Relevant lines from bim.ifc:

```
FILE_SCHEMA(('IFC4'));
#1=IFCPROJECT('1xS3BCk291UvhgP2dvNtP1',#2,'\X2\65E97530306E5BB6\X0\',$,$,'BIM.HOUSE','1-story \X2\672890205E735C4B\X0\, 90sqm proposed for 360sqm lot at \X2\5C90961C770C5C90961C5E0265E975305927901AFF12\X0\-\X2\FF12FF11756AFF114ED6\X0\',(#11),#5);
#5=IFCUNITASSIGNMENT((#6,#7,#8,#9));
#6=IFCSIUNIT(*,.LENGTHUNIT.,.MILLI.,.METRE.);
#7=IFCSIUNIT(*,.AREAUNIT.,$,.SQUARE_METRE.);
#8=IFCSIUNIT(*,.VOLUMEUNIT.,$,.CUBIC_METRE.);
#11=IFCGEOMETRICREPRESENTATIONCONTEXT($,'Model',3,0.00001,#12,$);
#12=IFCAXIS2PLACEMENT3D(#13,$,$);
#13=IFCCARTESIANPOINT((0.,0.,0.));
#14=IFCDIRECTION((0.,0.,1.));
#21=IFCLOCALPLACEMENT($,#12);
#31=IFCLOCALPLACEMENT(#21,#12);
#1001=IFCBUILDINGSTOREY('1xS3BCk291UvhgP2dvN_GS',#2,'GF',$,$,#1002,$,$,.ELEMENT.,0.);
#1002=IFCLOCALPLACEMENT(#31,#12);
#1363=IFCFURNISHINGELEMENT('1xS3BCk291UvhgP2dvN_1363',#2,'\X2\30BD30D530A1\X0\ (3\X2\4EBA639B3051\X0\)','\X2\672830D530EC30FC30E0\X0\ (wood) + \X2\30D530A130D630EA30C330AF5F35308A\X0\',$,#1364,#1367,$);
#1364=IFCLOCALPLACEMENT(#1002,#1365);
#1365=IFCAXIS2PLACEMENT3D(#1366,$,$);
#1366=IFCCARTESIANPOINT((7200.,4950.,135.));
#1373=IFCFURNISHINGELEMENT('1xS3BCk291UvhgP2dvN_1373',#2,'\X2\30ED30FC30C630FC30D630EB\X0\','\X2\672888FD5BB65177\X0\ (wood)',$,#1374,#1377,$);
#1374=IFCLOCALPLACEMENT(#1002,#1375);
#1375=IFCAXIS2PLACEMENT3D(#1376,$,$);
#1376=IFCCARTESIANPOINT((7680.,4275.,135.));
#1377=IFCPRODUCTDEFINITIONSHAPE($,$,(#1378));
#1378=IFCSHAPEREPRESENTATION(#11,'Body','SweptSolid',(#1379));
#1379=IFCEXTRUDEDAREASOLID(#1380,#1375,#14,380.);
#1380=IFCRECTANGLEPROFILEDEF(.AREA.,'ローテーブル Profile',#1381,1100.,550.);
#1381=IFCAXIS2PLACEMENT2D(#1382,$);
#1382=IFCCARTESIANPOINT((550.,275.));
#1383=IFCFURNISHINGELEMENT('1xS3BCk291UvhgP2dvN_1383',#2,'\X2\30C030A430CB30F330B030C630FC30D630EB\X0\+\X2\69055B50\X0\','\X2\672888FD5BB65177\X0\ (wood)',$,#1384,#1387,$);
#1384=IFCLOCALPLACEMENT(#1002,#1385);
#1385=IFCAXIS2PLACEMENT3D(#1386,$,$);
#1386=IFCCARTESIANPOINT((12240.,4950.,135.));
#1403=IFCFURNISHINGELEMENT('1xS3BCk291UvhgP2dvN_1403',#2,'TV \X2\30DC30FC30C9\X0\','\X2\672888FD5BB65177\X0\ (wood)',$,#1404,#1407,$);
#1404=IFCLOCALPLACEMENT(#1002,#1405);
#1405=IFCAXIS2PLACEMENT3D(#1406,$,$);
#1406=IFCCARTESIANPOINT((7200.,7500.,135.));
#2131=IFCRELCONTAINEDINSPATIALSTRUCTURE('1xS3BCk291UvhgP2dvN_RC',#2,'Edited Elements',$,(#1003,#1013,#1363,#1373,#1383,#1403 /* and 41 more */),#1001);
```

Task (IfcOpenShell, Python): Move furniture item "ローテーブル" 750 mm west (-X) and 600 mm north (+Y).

```python
import ifcopenshell
import ifcopenshell.api.geometry
import ifcopenshell.util.placement
import ifcopenshell.util.unit

model = ifcopenshell.open("bim.ifc")
unit_scale = ifcopenshell.util.unit.calculate_unit_scale(model)

item = model.by_guid("1xS3BCk291UvhgP2dvN_1373")
matrix = ifcopenshell.util.placement.get_local_placement(item.ObjectPlacement)
matrix[0, 3] -= 0.75 / unit_scale
matrix[1, 3] += 0.6 / unit_scale
ifcopenshell.api.geometry.edit_object_placement(model, product=item, matrix=matrix, is_si=False)

print(ifcopenshell.util.placement.get_local_placement(item.ObjectPlacement).round(3) + 0.0)

model.write("bim_updated.ifc")
```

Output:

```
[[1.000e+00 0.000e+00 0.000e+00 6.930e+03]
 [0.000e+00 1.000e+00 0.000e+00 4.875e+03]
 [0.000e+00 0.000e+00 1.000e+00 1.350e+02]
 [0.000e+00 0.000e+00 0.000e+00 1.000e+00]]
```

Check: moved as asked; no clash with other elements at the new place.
